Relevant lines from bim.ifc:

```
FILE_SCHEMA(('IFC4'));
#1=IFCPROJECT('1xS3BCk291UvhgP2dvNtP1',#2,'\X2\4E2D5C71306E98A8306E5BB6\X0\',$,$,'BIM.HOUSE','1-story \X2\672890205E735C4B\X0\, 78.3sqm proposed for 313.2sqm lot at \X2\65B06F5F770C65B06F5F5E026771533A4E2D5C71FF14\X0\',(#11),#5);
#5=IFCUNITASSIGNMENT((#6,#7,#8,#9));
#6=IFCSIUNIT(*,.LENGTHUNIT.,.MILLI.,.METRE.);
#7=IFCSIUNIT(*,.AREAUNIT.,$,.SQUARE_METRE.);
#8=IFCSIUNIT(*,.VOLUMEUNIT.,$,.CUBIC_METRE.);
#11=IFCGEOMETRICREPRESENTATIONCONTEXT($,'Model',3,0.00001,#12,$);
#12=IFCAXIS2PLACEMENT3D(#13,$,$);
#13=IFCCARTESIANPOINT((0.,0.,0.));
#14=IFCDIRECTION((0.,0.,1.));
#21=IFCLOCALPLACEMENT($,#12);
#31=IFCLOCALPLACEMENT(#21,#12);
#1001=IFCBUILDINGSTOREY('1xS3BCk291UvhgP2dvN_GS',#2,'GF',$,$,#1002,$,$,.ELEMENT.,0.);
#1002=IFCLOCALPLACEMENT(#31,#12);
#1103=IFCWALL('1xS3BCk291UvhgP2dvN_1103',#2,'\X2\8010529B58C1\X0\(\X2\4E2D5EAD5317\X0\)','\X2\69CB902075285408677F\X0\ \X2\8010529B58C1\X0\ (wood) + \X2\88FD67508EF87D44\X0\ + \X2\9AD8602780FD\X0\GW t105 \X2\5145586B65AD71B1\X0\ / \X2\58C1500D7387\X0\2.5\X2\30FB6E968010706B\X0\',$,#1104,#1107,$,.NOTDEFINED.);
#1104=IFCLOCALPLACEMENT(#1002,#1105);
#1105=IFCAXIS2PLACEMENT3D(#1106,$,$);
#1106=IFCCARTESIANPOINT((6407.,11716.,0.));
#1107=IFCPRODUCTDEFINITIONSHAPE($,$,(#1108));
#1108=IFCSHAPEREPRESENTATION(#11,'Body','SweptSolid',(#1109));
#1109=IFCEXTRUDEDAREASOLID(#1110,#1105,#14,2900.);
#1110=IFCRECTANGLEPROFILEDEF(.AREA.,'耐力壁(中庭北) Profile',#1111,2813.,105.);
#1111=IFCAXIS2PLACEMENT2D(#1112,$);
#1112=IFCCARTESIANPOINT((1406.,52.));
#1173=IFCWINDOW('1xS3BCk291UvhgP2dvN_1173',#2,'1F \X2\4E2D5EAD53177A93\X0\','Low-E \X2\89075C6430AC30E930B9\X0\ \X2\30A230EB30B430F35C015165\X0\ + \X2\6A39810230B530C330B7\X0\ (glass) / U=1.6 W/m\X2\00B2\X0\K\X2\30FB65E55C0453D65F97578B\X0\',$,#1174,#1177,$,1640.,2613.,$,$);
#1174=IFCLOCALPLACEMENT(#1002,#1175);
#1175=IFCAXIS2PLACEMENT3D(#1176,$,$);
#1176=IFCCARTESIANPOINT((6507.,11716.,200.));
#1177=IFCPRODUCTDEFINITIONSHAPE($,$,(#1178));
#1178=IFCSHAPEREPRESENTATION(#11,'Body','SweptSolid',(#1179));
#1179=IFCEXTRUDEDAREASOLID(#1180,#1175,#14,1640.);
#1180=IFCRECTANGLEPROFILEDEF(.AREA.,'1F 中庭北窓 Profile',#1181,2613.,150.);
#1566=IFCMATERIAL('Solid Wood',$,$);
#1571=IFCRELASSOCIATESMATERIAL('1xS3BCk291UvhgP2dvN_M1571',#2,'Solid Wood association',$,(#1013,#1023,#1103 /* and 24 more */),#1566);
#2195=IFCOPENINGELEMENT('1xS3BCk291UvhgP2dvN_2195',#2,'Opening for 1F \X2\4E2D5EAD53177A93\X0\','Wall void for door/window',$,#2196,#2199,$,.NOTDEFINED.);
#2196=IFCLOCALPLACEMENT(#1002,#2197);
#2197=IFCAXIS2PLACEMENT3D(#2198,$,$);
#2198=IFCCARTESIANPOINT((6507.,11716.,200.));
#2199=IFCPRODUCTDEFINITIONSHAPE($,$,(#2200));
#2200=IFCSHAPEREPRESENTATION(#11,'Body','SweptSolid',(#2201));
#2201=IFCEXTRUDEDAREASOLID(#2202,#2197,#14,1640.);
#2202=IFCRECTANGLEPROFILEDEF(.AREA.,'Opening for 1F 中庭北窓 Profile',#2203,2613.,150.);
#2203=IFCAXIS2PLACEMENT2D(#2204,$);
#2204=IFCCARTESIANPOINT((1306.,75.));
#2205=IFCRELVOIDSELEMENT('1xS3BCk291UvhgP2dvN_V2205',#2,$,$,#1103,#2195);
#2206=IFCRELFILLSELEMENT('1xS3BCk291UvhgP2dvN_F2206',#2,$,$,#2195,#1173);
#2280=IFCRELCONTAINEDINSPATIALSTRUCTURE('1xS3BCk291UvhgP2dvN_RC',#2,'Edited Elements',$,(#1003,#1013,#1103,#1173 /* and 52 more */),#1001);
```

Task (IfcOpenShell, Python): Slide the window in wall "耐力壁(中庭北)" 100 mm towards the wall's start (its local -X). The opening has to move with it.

```python
import ifcopenshell
import ifcopenshell.api.geometry
import ifcopenshell.util.placement
import ifcopenshell.util.unit

model = ifcopenshell.open("bim.ifc")
unit_scale = ifcopenshell.util.unit.calculate_unit_scale(model)

window = model.by_guid("1xS3BCk291UvhgP2dvN_1173")
opening = window.FillsVoids[0].RelatingOpeningElement
wall = opening.VoidsElements[0].RelatingBuildingElement

wall_matrix = ifcopenshell.util.placement.get_local_placement(wall.ObjectPlacement)
shift = wall_matrix[:3, 0] * -0.1 / unit_scale
before = ifcopenshell.util.placement.get_local_placement(window.ObjectPlacement)[:3, 3].copy()

# The window is not placed relative to its opening, so move both.
for product in (opening, window):
    matrix = ifcopenshell.util.placement.get_local_placement(product.ObjectPlacement)
    matrix[:3, 3] += shift
    ifcopenshell.api.geometry.edit_object_placement(model, product=product, matrix=matrix, is_si=False)

after = ifcopenshell.util.placement.get_local_placement(window.ObjectPlacement)[:3, 3]
print("window moved by", (after - before).round(3) + 0.0)

model.write("bim_v2.ifc")
```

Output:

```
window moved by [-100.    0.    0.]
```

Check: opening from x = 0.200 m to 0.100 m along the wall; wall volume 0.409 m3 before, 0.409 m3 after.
